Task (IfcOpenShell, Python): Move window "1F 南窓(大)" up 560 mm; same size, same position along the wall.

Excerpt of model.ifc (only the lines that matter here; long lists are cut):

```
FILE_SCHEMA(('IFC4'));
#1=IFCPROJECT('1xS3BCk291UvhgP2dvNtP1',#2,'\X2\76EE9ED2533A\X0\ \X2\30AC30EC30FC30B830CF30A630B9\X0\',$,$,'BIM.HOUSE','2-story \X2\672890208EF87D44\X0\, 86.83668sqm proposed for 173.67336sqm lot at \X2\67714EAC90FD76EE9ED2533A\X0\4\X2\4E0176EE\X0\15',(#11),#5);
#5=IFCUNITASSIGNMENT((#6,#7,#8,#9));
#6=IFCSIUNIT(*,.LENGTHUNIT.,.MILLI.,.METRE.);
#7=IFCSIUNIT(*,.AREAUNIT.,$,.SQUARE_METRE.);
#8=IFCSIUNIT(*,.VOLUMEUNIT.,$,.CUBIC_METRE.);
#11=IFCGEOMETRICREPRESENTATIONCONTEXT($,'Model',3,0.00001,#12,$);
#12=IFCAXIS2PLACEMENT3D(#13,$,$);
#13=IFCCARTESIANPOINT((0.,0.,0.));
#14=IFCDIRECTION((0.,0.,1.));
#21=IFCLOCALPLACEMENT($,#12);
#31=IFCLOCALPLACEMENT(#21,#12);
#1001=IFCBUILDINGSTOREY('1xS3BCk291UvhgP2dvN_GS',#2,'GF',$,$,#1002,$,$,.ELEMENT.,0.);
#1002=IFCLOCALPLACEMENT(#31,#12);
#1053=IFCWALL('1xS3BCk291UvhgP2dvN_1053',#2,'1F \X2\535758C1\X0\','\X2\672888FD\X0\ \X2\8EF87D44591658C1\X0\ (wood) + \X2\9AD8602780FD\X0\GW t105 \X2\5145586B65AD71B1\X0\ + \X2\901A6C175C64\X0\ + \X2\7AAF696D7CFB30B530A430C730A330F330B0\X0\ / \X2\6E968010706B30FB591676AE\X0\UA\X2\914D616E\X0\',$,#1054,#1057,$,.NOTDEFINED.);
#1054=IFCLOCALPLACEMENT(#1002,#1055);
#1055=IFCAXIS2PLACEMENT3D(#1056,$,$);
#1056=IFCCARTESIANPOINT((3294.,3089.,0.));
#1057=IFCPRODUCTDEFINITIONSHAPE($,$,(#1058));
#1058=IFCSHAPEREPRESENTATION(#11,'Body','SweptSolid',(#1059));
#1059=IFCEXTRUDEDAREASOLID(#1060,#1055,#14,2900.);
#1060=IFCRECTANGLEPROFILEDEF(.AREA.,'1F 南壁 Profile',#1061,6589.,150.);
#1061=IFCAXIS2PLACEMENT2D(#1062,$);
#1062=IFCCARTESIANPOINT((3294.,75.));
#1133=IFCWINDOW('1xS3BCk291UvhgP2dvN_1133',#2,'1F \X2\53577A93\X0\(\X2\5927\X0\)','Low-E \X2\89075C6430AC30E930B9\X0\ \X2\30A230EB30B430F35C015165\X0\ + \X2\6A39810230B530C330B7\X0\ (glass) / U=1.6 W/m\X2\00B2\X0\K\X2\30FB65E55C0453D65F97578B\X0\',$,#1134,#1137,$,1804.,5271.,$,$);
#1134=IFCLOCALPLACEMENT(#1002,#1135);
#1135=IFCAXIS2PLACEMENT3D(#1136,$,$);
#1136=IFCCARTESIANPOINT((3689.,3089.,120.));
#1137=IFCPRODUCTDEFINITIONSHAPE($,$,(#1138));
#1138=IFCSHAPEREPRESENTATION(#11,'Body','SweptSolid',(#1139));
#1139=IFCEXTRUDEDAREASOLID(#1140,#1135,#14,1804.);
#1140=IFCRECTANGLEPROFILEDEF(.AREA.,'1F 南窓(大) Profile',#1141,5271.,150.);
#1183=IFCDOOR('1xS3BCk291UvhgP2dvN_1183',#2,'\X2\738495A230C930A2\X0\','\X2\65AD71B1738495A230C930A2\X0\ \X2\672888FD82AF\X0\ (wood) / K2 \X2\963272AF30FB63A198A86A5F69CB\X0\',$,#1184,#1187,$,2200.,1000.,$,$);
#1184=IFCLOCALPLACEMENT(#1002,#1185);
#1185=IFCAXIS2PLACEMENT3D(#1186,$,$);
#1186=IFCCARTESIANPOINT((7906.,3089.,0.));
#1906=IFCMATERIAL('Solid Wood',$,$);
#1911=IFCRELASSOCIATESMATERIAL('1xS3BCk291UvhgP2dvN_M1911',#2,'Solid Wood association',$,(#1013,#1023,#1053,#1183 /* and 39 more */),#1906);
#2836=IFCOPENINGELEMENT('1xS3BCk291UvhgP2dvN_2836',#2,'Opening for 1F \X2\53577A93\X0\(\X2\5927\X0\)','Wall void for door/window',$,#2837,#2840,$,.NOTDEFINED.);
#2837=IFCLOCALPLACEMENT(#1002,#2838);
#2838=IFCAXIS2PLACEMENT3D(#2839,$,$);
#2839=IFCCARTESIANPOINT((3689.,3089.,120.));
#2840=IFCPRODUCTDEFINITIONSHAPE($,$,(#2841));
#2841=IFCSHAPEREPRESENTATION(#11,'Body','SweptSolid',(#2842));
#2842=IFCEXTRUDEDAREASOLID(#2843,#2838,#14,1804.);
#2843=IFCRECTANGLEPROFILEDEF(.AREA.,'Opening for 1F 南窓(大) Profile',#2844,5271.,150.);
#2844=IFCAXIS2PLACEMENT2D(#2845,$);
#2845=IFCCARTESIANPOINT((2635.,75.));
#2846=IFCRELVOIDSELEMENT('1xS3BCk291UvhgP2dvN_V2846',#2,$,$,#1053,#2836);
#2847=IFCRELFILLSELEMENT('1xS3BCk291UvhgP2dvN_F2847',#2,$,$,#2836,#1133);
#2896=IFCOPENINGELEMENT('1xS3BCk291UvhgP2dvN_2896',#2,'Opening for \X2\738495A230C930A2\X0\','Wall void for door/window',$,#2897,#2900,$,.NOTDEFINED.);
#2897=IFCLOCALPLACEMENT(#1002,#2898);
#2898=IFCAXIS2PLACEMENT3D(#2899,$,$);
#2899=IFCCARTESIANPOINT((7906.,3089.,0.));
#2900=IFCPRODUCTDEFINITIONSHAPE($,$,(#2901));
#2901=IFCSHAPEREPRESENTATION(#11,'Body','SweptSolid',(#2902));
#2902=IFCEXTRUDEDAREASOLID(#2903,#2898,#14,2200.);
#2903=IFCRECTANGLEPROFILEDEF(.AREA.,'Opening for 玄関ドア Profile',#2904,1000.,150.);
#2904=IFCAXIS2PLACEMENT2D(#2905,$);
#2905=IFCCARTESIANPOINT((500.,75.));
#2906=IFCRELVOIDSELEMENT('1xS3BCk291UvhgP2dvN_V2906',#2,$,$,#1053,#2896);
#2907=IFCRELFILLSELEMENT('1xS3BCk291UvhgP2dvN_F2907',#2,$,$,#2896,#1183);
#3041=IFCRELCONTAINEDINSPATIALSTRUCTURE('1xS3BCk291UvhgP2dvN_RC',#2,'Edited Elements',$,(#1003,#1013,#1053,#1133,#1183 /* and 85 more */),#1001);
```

```python
import numpy as np
import ifcopenshell
import ifcopenshell.api.geometry
import ifcopenshell.util.placement
import ifcopenshell.util.unit

model = ifcopenshell.open("model.ifc")
unit_scale = ifcopenshell.util.unit.calculate_unit_scale(model)

window = model.by_guid("1xS3BCk291UvhgP2dvN_1133")
opening = window.FillsVoids[0].RelatingOpeningElement
dz = 0.56 / unit_scale

shift = np.array([0.0, 0.0, dz])
# The window is not placed relative to its opening, so move both.
for product in (opening, window):
    matrix = ifcopenshell.util.placement.get_local_placement(product.ObjectPlacement)
    matrix[:3, 3] += shift
    ifcopenshell.api.geometry.edit_object_placement(model, product=product, matrix=matrix, is_si=False)

print(f"moved by {dz * unit_scale:+.3f} m")

model.write("model_edited.ifc")
```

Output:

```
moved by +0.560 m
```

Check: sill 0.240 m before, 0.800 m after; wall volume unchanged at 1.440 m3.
